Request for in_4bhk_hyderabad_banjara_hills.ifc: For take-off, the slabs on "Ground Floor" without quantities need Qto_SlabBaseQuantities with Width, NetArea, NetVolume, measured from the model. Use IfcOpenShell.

First a look at what the model holds.

```python
import ifcopenshell
import ifcopenshell.util.element
import ifcopenshell.util.unit

model = ifcopenshell.open("in_4bhk_hyderabad_banjara_hills.ifc")
print(model.schema)
for unit_type in ("LENGTHUNIT", "AREAUNIT", "VOLUMEUNIT"):
    print(unit_type, ifcopenshell.util.unit.calculate_unit_scale(model, unit_type))
storey = next(s for s in model.by_type("IfcBuildingStorey") if s.Name == "Ground Floor")
slabs = [e for e in ifcopenshell.util.element.get_decomposition(storey) if e.is_a("IfcSlab")]
for e in sorted(slabs, key=lambda e: e.id()):
    print(e.id(), e.is_a(), e.Name, list(ifcopenshell.util.element.get_psets(e, qtos_only=True)), sep=" | ")
```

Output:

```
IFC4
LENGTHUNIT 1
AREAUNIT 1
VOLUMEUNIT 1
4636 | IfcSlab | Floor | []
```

```python
import ifcopenshell
import ifcopenshell.api.pset
import ifcopenshell.geom
import ifcopenshell.util.element
import ifcopenshell.util.shape
import ifcopenshell.util.unit

model = ifcopenshell.open("in_4bhk_hyderabad_banjara_hills.ifc")
unit_scale = ifcopenshell.util.unit.calculate_unit_scale(model)
area_scale = ifcopenshell.util.unit.calculate_unit_scale(model, "AREAUNIT")
volume_scale = ifcopenshell.util.unit.calculate_unit_scale(model, "VOLUMEUNIT")
settings = ifcopenshell.geom.settings()

storey = next(s for s in model.by_type("IfcBuildingStorey") if s.Name == "Ground Floor")
slabs = [e for e in ifcopenshell.util.element.get_decomposition(storey) if e.is_a("IfcSlab")]

for e in sorted(slabs, key=lambda e: e.id()):
    if ifcopenshell.util.element.get_psets(e, qtos_only=True, should_inherit=False):
        continue
    # Geometry comes back in metres, in the element's own axes.
    shape = ifcopenshell.geom.create_shape(settings, e)
    values = {
        "Width": ifcopenshell.util.shape.get_z(shape.geometry) / unit_scale,
        "NetArea": ifcopenshell.util.shape.get_footprint_area(shape.geometry) / area_scale,
        "NetVolume": ifcopenshell.util.shape.get_volume(shape.geometry) / volume_scale,
    }
    qto = ifcopenshell.api.pset.add_qto(model, product=e, name="Qto_SlabBaseQuantities")
    ifcopenshell.api.pset.edit_qto(model, qto=qto, properties=values)
    print(e.id(), {k: round(v, 3) for k, v in values.items()})

model.write("in_4bhk_hyderabad_banjara_hills_rev.ifc")
```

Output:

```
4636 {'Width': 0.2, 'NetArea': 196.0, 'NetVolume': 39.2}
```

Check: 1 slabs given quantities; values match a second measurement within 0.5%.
